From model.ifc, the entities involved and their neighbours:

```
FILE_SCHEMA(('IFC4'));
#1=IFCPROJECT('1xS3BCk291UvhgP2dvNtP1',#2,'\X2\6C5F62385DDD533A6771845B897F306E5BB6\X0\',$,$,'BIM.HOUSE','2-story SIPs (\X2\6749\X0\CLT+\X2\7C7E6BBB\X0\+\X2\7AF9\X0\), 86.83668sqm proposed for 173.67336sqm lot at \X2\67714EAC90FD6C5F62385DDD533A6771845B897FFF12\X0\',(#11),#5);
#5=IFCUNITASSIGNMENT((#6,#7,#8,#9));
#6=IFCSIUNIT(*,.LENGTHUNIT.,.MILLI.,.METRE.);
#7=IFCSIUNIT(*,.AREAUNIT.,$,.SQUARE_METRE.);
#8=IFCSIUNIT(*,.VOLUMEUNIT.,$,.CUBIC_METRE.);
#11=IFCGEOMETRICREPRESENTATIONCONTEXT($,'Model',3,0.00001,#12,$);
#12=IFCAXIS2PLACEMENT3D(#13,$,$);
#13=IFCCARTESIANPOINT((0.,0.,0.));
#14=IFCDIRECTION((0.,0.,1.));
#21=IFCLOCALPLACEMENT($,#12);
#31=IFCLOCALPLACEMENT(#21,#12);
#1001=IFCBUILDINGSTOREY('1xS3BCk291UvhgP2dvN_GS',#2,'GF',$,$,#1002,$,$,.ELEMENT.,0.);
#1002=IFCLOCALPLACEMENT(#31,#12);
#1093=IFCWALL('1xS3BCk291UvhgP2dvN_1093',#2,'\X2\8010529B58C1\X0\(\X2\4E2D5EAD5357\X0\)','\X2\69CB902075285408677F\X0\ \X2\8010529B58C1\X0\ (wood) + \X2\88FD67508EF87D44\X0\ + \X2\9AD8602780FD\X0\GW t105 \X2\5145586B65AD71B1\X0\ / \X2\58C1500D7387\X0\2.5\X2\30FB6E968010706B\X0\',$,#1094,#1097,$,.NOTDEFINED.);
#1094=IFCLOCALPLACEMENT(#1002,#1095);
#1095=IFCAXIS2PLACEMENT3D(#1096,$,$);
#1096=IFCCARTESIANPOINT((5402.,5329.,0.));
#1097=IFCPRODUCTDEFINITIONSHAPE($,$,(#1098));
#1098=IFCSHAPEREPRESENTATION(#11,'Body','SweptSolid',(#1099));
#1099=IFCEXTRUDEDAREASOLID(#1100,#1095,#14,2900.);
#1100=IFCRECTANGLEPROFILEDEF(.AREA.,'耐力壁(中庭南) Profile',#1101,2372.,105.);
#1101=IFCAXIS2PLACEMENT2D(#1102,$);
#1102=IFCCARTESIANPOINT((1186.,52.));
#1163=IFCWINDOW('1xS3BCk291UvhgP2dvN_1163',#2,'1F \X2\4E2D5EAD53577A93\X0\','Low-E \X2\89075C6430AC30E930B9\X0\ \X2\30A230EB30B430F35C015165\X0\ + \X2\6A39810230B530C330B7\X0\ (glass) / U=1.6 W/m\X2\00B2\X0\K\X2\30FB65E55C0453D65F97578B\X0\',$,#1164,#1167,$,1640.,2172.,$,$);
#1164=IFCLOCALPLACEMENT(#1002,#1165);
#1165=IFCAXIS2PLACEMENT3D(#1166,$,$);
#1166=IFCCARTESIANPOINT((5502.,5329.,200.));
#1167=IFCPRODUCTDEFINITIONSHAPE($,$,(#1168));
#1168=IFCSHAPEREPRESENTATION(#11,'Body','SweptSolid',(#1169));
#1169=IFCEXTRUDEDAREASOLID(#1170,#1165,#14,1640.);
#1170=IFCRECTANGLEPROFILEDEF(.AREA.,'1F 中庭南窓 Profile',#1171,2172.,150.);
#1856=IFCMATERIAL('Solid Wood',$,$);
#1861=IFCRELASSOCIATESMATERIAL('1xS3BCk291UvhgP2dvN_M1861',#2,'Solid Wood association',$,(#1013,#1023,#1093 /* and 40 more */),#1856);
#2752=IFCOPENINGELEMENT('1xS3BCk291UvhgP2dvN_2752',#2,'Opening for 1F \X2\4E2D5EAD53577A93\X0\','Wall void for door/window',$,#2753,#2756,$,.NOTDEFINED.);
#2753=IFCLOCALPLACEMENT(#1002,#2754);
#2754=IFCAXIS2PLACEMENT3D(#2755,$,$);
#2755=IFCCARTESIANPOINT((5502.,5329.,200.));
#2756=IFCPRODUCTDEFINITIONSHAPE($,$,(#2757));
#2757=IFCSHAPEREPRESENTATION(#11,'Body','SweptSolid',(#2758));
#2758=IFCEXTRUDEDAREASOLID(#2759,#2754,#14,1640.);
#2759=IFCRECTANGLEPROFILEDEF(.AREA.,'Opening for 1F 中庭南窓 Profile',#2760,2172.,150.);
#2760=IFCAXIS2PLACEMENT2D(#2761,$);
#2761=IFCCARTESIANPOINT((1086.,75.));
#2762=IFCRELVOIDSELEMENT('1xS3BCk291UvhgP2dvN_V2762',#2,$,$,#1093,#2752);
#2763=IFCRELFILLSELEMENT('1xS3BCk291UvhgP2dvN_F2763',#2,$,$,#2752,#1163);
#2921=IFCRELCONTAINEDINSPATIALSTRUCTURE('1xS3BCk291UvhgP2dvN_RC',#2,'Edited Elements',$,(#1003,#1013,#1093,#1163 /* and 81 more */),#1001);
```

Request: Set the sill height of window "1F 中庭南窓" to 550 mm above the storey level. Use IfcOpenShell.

```python
import numpy as np
import ifcopenshell
import ifcopenshell.api.geometry
import ifcopenshell.geom
import ifcopenshell.util.element
import ifcopenshell.util.placement
import ifcopenshell.util.shape
import ifcopenshell.util.unit

model = ifcopenshell.open("model.ifc")
unit_scale = ifcopenshell.util.unit.calculate_unit_scale(model)

window = model.by_id(1163)
opening = window.FillsVoids[0].RelatingOpeningElement
storey = ifcopenshell.util.element.get_container(window, ifc_class="IfcBuildingStorey")
level = ifcopenshell.util.placement.get_local_placement(storey.ObjectPlacement)[2, 3]

# The opening's origin need not be at the sill, so measure its lowest point.
shape = ifcopenshell.geom.create_shape(ifcopenshell.geom.settings(), opening)
bottom = ifcopenshell.util.shape.get_shape_bottom_elevation(shape, shape.geometry) / unit_scale
dz = level + 0.55 / unit_scale - bottom

shift = np.array([0.0, 0.0, dz])
# The window is not placed relative to its opening, so move both.
for product in (opening, window):
    matrix = ifcopenshell.util.placement.get_local_placement(product.ObjectPlacement)
    matrix[:3, 3] += shift
    ifcopenshell.api.geometry.edit_object_placement(model, product=product, matrix=matrix, is_si=False)

print(f"moved by {dz * unit_scale:+.3f} m")

model.write("model_updated.ifc")
```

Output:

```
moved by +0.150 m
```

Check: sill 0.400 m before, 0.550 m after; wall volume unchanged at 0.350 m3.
